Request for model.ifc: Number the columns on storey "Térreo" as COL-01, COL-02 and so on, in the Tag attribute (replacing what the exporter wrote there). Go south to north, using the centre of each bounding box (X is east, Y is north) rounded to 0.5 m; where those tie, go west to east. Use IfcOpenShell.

First a look at what the model holds.

```python
import ifcopenshell
import ifcopenshell.util.element
import ifcopenshell.util.placement

model = ifcopenshell.open("model.ifc")
print(model.schema)
storey = next(s for s in model.by_type("IfcBuildingStorey") if s.Name == "Térreo")
columns = [e for e in ifcopenshell.util.element.get_decomposition(storey) if e.is_a("IfcColumn")]
for e in sorted(columns, key=lambda e: e.id()):
    origin = ifcopenshell.util.placement.get_local_placement(e.ObjectPlacement)[:3, 3]
    print(e.id(), e.Tag, e.Name, origin.round(2) + 0.0, sep=" | ")
```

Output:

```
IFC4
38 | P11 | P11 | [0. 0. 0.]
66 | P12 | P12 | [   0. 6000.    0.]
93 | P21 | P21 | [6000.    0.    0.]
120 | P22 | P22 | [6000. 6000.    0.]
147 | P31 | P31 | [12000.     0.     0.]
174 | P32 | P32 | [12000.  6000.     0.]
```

```python
import ifcopenshell
import ifcopenshell.geom
import ifcopenshell.util.element
import ifcopenshell.util.shape

model = ifcopenshell.open("model.ifc")
settings = ifcopenshell.geom.settings()
settings.set("use-world-coords", True)


def centre(element):
    shape = ifcopenshell.geom.create_shape(settings, element)
    return ifcopenshell.util.shape.get_bbox_centroid(shape.geometry)


storey = next(s for s in model.by_type("IfcBuildingStorey") if s.Name == "Térreo")
columns = [e for e in ifcopenshell.util.element.get_decomposition(storey) if e.is_a("IfcColumn")]

# Insertion points can sit at a corner or the storey origin, so sort by the geometry (in metres).
centres = {e: centre(e) for e in columns}
columns.sort(key=lambda e: (round(centres[e][1] / 0.5), centres[e][0]))

for i, e in enumerate(columns, start=1):
    number = f"COL-{i:02d}"
    e.Tag = number
    print(e.id(), number)

model.write("model_v2.ifc")
```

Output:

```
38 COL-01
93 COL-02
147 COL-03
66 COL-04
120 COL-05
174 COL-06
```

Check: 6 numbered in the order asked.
